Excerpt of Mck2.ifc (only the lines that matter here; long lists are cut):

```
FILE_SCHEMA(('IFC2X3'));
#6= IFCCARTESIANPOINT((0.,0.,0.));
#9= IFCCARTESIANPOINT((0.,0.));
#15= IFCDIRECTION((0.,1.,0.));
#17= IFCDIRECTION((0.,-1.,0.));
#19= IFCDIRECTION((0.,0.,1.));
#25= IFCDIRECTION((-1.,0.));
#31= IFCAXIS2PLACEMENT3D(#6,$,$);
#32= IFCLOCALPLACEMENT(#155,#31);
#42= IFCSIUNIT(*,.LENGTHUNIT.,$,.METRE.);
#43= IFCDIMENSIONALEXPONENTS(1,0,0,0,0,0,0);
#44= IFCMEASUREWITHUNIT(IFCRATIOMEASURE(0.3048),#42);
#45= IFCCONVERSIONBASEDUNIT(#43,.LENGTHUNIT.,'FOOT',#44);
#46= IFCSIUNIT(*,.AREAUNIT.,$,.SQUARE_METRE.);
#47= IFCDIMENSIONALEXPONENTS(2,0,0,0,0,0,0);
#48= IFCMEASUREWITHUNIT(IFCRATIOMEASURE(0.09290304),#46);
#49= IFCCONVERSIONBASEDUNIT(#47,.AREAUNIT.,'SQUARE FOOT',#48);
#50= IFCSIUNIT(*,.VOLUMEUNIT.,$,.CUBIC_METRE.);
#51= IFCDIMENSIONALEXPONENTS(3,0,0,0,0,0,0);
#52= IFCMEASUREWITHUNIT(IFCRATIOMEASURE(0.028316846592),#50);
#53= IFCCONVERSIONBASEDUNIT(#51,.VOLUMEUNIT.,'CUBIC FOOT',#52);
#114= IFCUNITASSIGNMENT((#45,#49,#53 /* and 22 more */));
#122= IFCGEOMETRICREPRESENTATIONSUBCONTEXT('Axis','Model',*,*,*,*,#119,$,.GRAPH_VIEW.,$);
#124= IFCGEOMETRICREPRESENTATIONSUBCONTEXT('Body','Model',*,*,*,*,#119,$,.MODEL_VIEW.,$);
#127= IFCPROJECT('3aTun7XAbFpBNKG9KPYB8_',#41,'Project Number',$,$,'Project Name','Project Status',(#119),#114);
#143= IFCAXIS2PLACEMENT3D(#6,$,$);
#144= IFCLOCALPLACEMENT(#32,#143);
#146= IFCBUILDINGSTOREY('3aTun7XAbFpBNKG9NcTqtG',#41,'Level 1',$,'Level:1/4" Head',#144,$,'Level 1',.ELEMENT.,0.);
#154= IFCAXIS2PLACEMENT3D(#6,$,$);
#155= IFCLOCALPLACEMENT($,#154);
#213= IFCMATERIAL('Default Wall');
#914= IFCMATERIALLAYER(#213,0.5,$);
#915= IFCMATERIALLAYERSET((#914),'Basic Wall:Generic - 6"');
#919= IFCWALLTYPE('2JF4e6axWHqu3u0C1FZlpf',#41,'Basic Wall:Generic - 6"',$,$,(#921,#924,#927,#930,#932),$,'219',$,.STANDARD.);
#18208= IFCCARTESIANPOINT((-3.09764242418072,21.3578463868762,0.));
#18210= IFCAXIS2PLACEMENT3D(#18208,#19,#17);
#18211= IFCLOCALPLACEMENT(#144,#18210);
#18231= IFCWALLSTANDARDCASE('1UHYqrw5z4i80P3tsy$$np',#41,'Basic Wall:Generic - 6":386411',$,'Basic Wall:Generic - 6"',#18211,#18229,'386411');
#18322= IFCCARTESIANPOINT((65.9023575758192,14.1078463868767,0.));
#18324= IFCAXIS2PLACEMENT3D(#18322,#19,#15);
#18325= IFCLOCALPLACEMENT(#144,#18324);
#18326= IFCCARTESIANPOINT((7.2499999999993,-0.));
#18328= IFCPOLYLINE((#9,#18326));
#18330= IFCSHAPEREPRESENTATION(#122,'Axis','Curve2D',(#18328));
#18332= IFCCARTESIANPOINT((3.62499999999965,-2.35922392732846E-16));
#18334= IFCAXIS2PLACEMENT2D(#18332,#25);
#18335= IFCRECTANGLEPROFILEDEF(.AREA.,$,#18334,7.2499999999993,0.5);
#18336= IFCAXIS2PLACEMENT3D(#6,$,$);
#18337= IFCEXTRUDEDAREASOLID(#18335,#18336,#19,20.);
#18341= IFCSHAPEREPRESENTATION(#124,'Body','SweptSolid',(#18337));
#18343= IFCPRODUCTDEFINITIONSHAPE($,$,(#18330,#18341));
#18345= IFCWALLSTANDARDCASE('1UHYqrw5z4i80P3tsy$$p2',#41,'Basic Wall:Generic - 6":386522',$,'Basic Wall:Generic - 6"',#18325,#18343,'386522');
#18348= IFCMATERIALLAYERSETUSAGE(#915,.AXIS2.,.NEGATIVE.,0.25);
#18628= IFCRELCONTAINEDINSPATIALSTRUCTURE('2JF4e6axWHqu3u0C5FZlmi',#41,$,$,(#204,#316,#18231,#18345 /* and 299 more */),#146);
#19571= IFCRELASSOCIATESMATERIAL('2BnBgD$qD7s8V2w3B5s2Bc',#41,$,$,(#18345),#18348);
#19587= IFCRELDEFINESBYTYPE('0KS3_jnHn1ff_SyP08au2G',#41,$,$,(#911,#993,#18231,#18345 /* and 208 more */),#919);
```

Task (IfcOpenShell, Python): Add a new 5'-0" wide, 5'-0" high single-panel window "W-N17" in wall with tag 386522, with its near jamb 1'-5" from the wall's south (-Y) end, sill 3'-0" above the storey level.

```python
import numpy as np
import ifcopenshell
import ifcopenshell.api.feature
import ifcopenshell.api.geometry
import ifcopenshell.api.root
import ifcopenshell.api.spatial
import ifcopenshell.api.type
import ifcopenshell.geom
import ifcopenshell.util.element
import ifcopenshell.util.placement
import ifcopenshell.util.representation
import ifcopenshell.util.shape
import ifcopenshell.util.unit

model = ifcopenshell.open("Mck2.ifc")
unit_scale = ifcopenshell.util.unit.calculate_unit_scale(model)
settings = ifcopenshell.geom.settings()


def volume(element):
    """Net volume in cubic metres, openings subtracted."""
    shape = ifcopenshell.geom.create_shape(settings, element)
    return ifcopenshell.util.shape.get_volume(shape.geometry)


wall = model.by_id(18345)
storey = ifcopenshell.util.element.get_container(wall, ifc_class="IfcBuildingStorey")
context = ifcopenshell.util.representation.get_context(model, "Model", "Body", "MODEL_VIEW")
before = volume(wall)

width, height, from_end, sill = 1.524, 1.524, 0.4318, 0.9144  # metres

# The wall runs along its own X axis, and the end named is its -X end.
wall_shape = ifcopenshell.geom.create_shape(settings, wall)
x, y, z = ifcopenshell.util.shape.get_vertices(wall_shape.geometry).T
start = x.min() + from_end
face, thickness = float(y.min()), float(y.max() - y.min())
wall_matrix = ifcopenshell.util.placement.get_local_placement(wall.ObjectPlacement)
level = ifcopenshell.util.placement.get_local_placement(storey.ObjectPlacement)[2, 3]


def in_wall(x, y):
    """Placement at x, y metres in the wall's axes, at sill height."""
    matrix = wall_matrix.copy()
    matrix[:, 3] = wall_matrix @ np.array([x / unit_scale, y / unit_scale, 0.0, 1.0])
    matrix[2, 3] = level + sill / unit_scale
    return matrix


# Opening: a box that overshoots both wall faces by 50 mm.
opening = ifcopenshell.api.root.create_entity(model, ifc_class="IfcOpeningElement")
box = ifcopenshell.api.geometry.add_wall_representation(
    model, context=context, length=width, height=height, thickness=thickness + 0.1
)
ifcopenshell.api.geometry.assign_representation(model, product=opening, representation=box)
ifcopenshell.api.geometry.edit_object_placement(model, product=opening, matrix=in_wall(start, face - 0.05), is_si=False)
ifcopenshell.api.feature.add_feature(model, feature=opening, element=wall)

window = ifcopenshell.api.root.create_entity(model, ifc_class="IfcWindow", name="W-N17")
window.OverallWidth, window.OverallHeight = width / unit_scale, height / unit_scale
body = ifcopenshell.api.geometry.add_window_representation(
    model,
    context=context,
    overall_width=window.OverallWidth,
    overall_height=window.OverallHeight,
    partition_type="SINGLE_PANEL",
)
ifcopenshell.api.geometry.assign_representation(model, product=window, representation=body)
ifcopenshell.api.spatial.assign_container(model, products=[window], relating_structure=storey)
fills = ifcopenshell.api.feature.add_filling(model, opening=opening, element=window)
fills.OwnerHistory = window.OwnerHistory  # required in IFC2X3

# IFC2X3 keeps the operation on the window style.
style = ifcopenshell.api.root.create_entity(model, ifc_class="IfcWindowStyle", name="W-N17")
style.OperationType, style.ConstructionType = "SINGLE_PANEL", "NOTDEFINED"
style.ParameterTakesPrecedence = style.Sizeable = False
ifcopenshell.api.type.assign_type(model, related_objects=[window], relating_type=style)

# Centre the window in the wall's thickness.
ifcopenshell.api.geometry.edit_object_placement(model, product=window, matrix=in_wall(start, face), is_si=False)
window_shape = ifcopenshell.geom.create_shape(settings, window)
depth = ifcopenshell.util.shape.get_vertices(window_shape.geometry)[:, 1]
offset = face + thickness / 2 - (depth.min() + depth.max()) / 2
ifcopenshell.api.geometry.edit_object_placement(model, product=window, matrix=in_wall(start, offset), is_si=False)

after = volume(wall)

print(f"wall volume {before:.3f} -> {after:.3f} m3")

model.write("Mck2-out.ifc")
```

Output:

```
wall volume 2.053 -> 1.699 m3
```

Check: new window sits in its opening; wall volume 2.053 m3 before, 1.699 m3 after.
